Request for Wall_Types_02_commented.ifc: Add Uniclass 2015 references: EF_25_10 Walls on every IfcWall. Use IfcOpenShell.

First a look at what the model holds.

```python
import ifcopenshell

model = ifcopenshell.open("Wall_Types_02_commented.ifc")
print(model.schema)
print("classifications:", [c.Name for c in model.by_type("IfcClassification")])
for ifc_class in ("IfcDoor", "IfcRoof", "IfcStair", "IfcWall", "IfcWindow"):
    print(ifc_class, len(model.by_type(ifc_class)))
```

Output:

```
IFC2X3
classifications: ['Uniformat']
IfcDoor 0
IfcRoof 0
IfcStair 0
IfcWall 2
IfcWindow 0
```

```python
import ifcopenshell
import ifcopenshell.api.classification

model = ifcopenshell.open("Wall_Types_02_commented.ifc")

# IFC2X3 requires Source and Edition and has no link from the project to the system.
system = model.create_entity("IfcClassification", Source="NBS", Edition="2015", Name="Uniclass 2015")

codes = {
    "IfcWall": ("EF_25_10", "Walls"),
}
for ifc_class, (code, name) in codes.items():
    products = model.by_type(ifc_class)
    ifcopenshell.api.classification.add_reference(
        model, products=products, classification=system, identification=code, name=name
    )
    print(code, len(products))

model.write("Wall_Types_02_commented_rev.ifc")
```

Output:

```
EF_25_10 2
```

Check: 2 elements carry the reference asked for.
